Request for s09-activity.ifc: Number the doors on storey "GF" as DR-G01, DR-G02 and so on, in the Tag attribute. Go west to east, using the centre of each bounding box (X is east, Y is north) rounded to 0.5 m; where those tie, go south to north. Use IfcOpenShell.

First a look at what the model holds.

```python
import ifcopenshell
import ifcopenshell.util.element
import ifcopenshell.util.placement

model = ifcopenshell.open("s09-activity.ifc")
print(model.schema)
storey = next(s for s in model.by_type("IfcBuildingStorey") if s.Name == "GF")
doors = [e for e in ifcopenshell.util.element.get_decomposition(storey) if e.is_a("IfcDoor")]
for e in sorted(doors, key=lambda e: e.id()):
    origin = ifcopenshell.util.placement.get_local_placement(e.ObjectPlacement)[:3, 3]
    print(e.id(), e.Tag, e.Name, origin.round(2) + 0.0, sep=" | ")
```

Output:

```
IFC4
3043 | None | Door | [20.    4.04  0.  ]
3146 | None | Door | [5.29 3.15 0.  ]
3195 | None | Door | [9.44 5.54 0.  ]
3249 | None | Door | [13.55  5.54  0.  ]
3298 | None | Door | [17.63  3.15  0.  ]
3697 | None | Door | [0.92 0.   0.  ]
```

```python
import ifcopenshell
import ifcopenshell.geom
import ifcopenshell.util.element
import ifcopenshell.util.shape

model = ifcopenshell.open("s09-activity.ifc")
settings = ifcopenshell.geom.settings()
settings.set("use-world-coords", True)


def centre(element):
    shape = ifcopenshell.geom.create_shape(settings, element)
    return ifcopenshell.util.shape.get_bbox_centroid(shape.geometry)


storey = next(s for s in model.by_type("IfcBuildingStorey") if s.Name == "GF")
doors = [e for e in ifcopenshell.util.element.get_decomposition(storey) if e.is_a("IfcDoor")]

# Insertion points can sit at a corner or the storey origin, so sort by the geometry (in metres).
centres = {e: centre(e) for e in doors}
doors.sort(key=lambda e: (round(centres[e][0] / 0.5), centres[e][1]))

for i, e in enumerate(doors, start=1):
    number = f"DR-G{i:02d}"
    e.Tag = number
    print(e.id(), number)

model.write("s09-activity_updated.ifc")
```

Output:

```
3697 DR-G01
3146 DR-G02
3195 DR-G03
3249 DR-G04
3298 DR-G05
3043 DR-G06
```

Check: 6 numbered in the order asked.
